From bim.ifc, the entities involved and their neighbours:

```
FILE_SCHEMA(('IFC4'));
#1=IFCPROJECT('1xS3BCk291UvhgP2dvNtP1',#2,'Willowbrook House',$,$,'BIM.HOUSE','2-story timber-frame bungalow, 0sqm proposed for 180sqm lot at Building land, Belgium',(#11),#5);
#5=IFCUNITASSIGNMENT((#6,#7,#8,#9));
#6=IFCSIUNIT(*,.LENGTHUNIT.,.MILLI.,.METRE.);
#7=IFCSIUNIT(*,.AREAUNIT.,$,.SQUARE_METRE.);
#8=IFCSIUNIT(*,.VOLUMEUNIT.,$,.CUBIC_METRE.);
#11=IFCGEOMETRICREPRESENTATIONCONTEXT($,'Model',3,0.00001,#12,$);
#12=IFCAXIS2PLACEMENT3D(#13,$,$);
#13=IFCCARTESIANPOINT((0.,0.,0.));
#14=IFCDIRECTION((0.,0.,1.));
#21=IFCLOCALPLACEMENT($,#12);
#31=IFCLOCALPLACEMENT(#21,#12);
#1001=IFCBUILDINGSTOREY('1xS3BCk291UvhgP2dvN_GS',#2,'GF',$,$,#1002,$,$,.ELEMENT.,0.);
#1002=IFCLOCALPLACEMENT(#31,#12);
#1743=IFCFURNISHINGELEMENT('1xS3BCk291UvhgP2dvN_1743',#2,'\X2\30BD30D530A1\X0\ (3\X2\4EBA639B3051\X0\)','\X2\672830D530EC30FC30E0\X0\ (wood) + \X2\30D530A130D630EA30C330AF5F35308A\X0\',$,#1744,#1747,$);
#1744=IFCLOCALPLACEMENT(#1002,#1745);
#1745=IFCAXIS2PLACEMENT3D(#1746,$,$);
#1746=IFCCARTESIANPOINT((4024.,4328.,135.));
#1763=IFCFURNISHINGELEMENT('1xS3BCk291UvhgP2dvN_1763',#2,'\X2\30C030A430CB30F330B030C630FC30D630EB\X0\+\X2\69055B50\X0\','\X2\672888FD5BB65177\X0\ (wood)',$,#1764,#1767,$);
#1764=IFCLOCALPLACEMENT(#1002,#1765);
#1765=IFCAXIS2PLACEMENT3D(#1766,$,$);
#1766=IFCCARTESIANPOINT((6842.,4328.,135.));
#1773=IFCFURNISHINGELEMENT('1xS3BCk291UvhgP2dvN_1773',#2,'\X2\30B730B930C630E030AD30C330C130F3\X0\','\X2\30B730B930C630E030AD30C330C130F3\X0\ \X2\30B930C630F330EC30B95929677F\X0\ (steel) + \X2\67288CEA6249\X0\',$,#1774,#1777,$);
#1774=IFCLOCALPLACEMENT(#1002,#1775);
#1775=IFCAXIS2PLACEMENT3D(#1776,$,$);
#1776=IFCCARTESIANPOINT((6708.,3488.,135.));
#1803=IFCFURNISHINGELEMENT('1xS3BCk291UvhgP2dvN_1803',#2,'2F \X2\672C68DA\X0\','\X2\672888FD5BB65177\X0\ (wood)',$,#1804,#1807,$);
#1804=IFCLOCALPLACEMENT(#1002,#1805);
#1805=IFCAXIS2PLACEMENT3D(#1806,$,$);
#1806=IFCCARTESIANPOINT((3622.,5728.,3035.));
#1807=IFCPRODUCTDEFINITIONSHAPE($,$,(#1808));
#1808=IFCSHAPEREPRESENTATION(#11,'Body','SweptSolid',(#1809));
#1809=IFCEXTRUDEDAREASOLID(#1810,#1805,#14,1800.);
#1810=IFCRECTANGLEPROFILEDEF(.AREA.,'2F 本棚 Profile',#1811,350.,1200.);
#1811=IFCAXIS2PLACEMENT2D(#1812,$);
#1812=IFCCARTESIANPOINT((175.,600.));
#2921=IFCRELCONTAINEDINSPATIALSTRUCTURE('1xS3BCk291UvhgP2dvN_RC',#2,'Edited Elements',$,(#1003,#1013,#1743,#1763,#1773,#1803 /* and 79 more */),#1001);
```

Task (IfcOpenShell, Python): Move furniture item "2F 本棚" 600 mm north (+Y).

```python
import ifcopenshell
import ifcopenshell.api.geometry
import ifcopenshell.util.placement
import ifcopenshell.util.unit

model = ifcopenshell.open("bim.ifc")
unit_scale = ifcopenshell.util.unit.calculate_unit_scale(model)

item = model.by_guid("1xS3BCk291UvhgP2dvN_1803")
matrix = ifcopenshell.util.placement.get_local_placement(item.ObjectPlacement)
matrix[1, 3] += 0.6 / unit_scale
ifcopenshell.api.geometry.edit_object_placement(model, product=item, matrix=matrix, is_si=False)

print(ifcopenshell.util.placement.get_local_placement(item.ObjectPlacement).round(3) + 0.0)

model.write("bim_rev.ifc")
```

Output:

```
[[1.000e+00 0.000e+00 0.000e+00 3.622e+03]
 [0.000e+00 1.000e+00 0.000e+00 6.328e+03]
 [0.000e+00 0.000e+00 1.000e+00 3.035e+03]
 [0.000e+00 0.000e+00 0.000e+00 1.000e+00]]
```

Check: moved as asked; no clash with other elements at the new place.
